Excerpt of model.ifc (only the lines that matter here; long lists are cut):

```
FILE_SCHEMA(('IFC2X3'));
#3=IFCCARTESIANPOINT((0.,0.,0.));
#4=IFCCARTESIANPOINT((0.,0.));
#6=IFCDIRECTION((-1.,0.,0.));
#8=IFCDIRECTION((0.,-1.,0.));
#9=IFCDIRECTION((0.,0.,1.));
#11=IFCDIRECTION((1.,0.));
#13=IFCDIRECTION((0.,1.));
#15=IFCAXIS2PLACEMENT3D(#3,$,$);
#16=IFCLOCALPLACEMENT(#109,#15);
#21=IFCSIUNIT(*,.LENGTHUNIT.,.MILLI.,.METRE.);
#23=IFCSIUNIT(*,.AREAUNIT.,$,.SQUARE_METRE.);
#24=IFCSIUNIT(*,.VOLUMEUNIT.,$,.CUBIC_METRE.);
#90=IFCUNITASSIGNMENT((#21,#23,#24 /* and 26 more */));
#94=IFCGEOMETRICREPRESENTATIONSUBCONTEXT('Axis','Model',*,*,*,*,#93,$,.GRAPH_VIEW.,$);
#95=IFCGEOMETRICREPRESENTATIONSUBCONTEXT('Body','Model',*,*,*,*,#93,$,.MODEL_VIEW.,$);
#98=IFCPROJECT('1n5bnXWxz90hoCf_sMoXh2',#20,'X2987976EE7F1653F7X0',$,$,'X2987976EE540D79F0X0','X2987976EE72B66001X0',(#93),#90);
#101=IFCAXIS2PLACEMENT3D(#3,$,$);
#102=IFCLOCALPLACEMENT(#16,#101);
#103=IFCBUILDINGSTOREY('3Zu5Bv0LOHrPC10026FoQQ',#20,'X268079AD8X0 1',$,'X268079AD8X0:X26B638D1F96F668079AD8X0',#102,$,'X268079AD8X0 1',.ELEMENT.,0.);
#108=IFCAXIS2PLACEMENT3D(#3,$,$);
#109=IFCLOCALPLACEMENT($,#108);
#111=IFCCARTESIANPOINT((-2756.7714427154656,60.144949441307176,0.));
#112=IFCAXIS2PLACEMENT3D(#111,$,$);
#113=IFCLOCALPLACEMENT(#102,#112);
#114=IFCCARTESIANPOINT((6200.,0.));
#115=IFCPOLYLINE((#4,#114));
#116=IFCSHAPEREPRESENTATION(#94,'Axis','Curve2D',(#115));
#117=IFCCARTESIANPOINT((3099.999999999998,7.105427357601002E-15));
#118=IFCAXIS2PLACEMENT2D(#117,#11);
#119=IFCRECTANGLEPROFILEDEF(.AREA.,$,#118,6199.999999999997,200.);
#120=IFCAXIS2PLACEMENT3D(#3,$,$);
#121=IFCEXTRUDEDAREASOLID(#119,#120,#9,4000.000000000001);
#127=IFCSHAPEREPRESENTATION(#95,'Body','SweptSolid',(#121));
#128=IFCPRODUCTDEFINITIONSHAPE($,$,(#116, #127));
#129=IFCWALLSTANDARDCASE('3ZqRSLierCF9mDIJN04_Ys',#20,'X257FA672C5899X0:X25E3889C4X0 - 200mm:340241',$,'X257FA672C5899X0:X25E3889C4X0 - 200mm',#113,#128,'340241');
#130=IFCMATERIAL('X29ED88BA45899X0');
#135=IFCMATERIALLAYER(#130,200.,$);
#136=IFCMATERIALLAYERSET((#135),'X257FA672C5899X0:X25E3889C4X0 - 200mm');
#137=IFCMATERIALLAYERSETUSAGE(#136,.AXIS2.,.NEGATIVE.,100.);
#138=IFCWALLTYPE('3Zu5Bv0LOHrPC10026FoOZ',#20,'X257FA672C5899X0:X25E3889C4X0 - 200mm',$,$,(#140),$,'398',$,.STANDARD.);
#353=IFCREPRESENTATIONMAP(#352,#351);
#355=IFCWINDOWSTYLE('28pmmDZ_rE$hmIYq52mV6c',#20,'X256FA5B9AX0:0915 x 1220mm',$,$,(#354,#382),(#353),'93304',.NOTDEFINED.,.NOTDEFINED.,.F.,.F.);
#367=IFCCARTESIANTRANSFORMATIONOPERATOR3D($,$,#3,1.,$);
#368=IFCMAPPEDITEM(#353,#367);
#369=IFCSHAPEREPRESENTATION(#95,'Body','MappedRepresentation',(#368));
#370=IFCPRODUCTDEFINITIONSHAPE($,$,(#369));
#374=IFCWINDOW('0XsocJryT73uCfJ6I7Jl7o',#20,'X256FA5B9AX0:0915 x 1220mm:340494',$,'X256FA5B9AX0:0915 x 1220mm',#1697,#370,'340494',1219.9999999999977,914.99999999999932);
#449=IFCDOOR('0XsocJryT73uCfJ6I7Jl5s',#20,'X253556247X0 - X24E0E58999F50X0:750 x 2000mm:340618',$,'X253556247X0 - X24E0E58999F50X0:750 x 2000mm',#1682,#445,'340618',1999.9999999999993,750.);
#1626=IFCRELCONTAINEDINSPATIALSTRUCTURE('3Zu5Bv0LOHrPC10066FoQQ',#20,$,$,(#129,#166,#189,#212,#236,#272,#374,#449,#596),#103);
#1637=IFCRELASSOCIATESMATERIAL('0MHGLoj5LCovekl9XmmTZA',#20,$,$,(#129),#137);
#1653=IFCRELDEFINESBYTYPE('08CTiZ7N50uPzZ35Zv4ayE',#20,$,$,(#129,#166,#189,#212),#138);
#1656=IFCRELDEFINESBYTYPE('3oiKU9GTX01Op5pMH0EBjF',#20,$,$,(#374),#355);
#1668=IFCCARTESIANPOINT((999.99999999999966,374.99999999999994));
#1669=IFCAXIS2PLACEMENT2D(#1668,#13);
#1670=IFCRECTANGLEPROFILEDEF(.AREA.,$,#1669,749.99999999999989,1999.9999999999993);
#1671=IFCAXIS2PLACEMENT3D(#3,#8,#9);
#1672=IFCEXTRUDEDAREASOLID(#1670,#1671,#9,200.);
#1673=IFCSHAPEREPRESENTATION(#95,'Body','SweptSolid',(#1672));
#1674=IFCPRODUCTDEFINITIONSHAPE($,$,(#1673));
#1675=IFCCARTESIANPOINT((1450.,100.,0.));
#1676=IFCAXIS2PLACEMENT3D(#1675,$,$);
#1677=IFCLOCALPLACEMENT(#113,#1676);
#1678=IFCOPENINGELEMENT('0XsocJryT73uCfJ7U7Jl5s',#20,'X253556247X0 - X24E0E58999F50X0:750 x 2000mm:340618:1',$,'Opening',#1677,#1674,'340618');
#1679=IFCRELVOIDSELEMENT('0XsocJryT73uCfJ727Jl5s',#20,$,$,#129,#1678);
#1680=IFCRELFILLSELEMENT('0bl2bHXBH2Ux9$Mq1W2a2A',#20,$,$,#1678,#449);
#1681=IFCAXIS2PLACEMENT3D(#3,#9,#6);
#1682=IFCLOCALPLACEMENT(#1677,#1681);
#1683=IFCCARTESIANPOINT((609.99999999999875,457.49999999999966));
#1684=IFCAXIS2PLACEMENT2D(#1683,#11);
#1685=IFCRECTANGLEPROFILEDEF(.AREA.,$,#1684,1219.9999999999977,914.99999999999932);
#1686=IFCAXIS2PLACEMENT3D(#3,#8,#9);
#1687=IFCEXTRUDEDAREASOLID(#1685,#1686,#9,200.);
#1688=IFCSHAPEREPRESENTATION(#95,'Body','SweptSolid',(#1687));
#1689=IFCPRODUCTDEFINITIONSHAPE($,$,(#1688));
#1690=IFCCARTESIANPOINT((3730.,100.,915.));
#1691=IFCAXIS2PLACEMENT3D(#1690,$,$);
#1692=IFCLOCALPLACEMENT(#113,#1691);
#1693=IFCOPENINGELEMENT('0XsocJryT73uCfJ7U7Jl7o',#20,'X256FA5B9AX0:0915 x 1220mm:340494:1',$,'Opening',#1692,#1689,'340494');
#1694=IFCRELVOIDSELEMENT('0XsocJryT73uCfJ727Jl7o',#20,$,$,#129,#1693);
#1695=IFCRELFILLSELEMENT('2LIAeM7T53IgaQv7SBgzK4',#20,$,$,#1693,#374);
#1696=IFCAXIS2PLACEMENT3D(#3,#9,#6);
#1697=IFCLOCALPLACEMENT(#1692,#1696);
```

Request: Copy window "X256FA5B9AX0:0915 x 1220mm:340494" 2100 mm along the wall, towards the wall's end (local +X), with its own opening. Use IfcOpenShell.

```python
import ifcopenshell
import ifcopenshell.api.feature
import ifcopenshell.api.geometry
import ifcopenshell.api.root
import ifcopenshell.geom
import ifcopenshell.util.element
import ifcopenshell.util.placement
import ifcopenshell.util.shape
import ifcopenshell.util.unit

model = ifcopenshell.open("model.ifc")
unit_scale = ifcopenshell.util.unit.calculate_unit_scale(model)
settings = ifcopenshell.geom.settings()


def volume(element):
    """Net volume in cubic metres, openings subtracted."""
    shape = ifcopenshell.geom.create_shape(settings, element)
    return ifcopenshell.util.shape.get_volume(shape.geometry)


def reuse_history(source, copy):
    """copy_class also copies each property set's owner history, people and application; keep the originals."""
    for rel in copy.IsDefinedBy:
        if rel.is_a("IfcRelDefinesByProperties") and (history := rel.RelatingPropertyDefinition.OwnerHistory):
            rel.RelatingPropertyDefinition.OwnerHistory = source.OwnerHistory
            ifcopenshell.util.element.remove_deep2(model, history)


window = model.by_guid("0XsocJryT73uCfJ6I7Jl7o")
opening = window.FillsVoids[0].RelatingOpeningElement
wall = opening.VoidsElements[0].RelatingBuildingElement
before = volume(wall)
shift = ifcopenshell.util.placement.get_local_placement(wall.ObjectPlacement)[:3, 0] * 2.1 / unit_scale

# copy_class copies the void relationship, type, container and properties, but no geometry.
new_opening = ifcopenshell.api.root.copy_class(model, product=opening)
new_opening.Representation = ifcopenshell.util.element.copy_deep(
    model, opening.Representation, exclude=["IfcGeometricRepresentationContext", "IfcRepresentationMap"]
)
new_opening.Name = "X256FA5B9AX0:0915 x 1220mm"
new_opening.Tag = None
new_window = ifcopenshell.api.root.copy_class(model, product=window)
new_window.Representation = ifcopenshell.util.element.copy_deep(
    model, window.Representation, exclude=["IfcGeometricRepresentationContext", "IfcRepresentationMap"]
)
new_window.Name = "X256FA5B9AX0:0915 x 1220mm"
new_window.Tag = None
reuse_history(window, new_window)
fills = ifcopenshell.api.feature.add_filling(model, opening=new_opening, element=new_window)
fills.OwnerHistory = new_window.OwnerHistory  # required in IFC2X3

for old, new in ((opening, new_opening), (window, new_window)):
    matrix = ifcopenshell.util.placement.get_local_placement(old.ObjectPlacement)
    matrix[:3, 3] += shift
    ifcopenshell.api.geometry.edit_object_placement(model, product=new, matrix=matrix, is_si=False)

after = volume(wall)

print(f"wall volume {before:.3f} -> {after:.3f} m3")

model.write("model_updated.ifc")
```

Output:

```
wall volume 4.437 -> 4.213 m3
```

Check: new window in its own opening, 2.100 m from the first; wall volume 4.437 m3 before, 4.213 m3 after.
